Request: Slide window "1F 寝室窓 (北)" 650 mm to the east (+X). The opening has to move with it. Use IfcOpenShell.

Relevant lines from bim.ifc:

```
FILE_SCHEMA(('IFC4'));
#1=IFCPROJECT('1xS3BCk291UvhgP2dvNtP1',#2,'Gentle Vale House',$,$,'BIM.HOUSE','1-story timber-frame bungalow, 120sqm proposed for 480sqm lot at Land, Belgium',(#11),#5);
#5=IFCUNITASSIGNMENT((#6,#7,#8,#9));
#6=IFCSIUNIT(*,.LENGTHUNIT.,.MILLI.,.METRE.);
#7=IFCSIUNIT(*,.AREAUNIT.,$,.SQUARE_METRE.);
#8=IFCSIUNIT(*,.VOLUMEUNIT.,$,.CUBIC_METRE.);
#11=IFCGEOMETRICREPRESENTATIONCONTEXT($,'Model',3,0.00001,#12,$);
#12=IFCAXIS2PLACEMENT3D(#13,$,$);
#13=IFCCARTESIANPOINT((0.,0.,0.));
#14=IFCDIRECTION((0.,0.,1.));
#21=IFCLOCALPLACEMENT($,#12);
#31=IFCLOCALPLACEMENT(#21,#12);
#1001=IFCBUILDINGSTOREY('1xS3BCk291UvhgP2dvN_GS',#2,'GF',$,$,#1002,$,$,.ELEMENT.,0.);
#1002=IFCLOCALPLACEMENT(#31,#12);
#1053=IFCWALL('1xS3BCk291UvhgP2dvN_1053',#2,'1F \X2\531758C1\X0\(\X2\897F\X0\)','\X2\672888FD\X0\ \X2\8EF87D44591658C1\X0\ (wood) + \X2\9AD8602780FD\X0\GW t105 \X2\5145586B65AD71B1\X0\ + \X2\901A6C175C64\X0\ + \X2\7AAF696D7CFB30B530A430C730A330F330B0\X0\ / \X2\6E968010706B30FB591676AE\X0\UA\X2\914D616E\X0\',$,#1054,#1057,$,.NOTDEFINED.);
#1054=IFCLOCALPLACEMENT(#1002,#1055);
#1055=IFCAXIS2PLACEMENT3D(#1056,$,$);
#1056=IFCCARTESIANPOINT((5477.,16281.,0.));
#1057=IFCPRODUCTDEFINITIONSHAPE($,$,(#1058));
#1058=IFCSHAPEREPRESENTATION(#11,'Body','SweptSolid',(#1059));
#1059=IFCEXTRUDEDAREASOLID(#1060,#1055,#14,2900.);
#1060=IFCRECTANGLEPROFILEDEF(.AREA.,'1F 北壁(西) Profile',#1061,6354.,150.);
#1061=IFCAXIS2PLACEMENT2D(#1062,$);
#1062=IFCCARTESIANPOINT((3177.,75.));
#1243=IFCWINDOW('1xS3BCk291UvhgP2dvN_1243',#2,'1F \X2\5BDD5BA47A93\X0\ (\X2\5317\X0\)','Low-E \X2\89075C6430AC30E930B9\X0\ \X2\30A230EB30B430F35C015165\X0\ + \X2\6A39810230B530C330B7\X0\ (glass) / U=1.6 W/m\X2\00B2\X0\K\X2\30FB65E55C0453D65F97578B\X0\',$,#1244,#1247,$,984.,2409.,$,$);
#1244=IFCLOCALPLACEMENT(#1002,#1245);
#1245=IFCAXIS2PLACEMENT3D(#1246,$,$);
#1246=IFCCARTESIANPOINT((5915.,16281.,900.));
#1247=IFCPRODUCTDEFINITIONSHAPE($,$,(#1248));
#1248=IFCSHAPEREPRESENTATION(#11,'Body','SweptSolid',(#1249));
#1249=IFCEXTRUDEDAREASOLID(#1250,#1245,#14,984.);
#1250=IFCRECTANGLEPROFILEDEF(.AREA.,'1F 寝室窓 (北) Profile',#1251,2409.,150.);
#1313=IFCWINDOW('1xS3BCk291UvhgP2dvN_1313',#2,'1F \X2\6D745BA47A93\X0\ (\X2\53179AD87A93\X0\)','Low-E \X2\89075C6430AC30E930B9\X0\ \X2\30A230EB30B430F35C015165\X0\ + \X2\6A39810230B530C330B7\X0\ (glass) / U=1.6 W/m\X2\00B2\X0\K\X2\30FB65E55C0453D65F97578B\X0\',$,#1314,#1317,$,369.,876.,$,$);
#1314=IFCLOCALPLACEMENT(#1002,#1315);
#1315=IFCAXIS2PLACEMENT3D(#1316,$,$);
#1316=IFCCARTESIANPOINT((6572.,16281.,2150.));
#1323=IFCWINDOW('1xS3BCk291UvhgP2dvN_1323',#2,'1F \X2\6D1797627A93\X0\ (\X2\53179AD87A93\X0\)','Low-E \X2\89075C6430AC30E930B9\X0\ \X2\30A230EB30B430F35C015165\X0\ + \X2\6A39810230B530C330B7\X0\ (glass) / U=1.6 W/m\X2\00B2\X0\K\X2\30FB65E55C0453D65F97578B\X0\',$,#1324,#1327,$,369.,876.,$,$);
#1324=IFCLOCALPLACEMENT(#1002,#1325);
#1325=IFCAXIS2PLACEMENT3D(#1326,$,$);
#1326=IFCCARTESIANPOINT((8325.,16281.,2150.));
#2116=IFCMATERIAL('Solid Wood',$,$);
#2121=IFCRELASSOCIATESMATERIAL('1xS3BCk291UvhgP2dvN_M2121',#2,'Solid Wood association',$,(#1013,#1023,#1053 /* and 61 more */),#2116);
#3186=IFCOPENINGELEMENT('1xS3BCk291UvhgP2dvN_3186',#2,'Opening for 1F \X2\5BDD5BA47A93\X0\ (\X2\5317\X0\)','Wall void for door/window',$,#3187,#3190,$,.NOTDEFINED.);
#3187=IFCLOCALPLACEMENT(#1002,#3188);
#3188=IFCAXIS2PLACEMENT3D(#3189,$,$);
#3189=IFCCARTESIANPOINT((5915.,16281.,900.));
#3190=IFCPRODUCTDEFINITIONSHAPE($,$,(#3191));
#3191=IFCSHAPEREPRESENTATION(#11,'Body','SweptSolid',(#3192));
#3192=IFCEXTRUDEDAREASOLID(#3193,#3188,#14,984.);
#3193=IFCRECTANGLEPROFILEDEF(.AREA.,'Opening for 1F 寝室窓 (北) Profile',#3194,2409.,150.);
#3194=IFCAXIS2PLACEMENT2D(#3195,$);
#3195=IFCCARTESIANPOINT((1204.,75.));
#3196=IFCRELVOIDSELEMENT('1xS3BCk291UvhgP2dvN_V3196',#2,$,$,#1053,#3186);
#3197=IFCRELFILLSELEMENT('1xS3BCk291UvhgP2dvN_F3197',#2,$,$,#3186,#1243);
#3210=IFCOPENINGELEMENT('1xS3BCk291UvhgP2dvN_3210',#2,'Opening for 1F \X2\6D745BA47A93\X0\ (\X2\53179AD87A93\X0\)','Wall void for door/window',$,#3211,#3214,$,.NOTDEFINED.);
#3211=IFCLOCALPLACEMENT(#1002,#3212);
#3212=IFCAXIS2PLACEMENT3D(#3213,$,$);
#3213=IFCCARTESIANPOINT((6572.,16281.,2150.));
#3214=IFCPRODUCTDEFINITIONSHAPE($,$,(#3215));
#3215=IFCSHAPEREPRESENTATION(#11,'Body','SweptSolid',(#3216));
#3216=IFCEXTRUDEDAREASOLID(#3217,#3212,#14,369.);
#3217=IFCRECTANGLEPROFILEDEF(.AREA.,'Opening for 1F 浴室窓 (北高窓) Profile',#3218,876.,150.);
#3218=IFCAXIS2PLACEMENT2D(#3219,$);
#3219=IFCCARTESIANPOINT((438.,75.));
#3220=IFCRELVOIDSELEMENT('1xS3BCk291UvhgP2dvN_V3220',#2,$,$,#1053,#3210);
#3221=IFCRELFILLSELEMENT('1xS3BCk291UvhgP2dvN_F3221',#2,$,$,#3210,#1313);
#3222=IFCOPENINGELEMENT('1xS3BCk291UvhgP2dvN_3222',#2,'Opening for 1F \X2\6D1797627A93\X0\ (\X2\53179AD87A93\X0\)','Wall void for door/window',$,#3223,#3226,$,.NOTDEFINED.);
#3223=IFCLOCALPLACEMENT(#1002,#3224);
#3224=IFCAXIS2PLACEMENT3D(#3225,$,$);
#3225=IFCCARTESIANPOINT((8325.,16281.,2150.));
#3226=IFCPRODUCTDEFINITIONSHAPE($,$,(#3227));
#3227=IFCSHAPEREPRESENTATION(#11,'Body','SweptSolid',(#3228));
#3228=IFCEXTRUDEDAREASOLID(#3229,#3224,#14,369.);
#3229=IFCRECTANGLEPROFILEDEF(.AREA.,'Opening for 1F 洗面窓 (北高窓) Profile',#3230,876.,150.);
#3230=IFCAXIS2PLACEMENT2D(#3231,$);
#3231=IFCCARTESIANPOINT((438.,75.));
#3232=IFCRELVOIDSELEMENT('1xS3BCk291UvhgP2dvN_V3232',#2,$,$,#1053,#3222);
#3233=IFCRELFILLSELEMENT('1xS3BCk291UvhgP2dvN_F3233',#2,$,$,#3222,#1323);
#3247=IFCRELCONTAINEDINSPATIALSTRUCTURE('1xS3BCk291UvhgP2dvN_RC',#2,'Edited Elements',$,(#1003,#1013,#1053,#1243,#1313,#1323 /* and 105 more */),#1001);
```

```python
import ifcopenshell
import ifcopenshell.api.geometry
import ifcopenshell.util.placement

model = ifcopenshell.open("bim.ifc")

window = model.by_id(1243)
opening = window.FillsVoids[0].RelatingOpeningElement
wall = opening.VoidsElements[0].RelatingBuildingElement

wall_matrix = ifcopenshell.util.placement.get_local_placement(wall.ObjectPlacement)
shift = wall_matrix[:3, 0] * 650.0
before = ifcopenshell.util.placement.get_local_placement(window.ObjectPlacement)[:3, 3].copy()

# The window is not placed relative to its opening, so move both.
for product in (opening, window):
    matrix = ifcopenshell.util.placement.get_local_placement(product.ObjectPlacement)
    matrix[:3, 3] += shift
    ifcopenshell.api.geometry.edit_object_placement(model, product=product, matrix=matrix, is_si=False)

after = ifcopenshell.util.placement.get_local_placement(window.ObjectPlacement)[:3, 3]
print("window moved by", (after - before).round(3) + 0.0)

model.write("bim_rev.ifc")
```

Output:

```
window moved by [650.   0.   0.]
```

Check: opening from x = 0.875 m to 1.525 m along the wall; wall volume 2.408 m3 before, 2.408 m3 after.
